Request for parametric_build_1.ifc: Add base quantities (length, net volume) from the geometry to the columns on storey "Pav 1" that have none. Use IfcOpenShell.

First a look at what the model holds.

```python
import ifcopenshell
import ifcopenshell.util.element
import ifcopenshell.util.unit

model = ifcopenshell.open("parametric_build_1.ifc")
print(model.schema)
for unit_type in ("LENGTHUNIT", "AREAUNIT", "VOLUMEUNIT"):
    print(unit_type, ifcopenshell.util.unit.calculate_unit_scale(model, unit_type))
storey = next(s for s in model.by_type("IfcBuildingStorey") if s.Name == "Pav 1")
columns = [e for e in ifcopenshell.util.element.get_decomposition(storey) if e.is_a("IfcColumn")]
for e in sorted(columns, key=lambda e: e.id()):
    print(e.id(), e.is_a(), e.Name, list(ifcopenshell.util.element.get_psets(e, qtos_only=True)), sep=" | ")
```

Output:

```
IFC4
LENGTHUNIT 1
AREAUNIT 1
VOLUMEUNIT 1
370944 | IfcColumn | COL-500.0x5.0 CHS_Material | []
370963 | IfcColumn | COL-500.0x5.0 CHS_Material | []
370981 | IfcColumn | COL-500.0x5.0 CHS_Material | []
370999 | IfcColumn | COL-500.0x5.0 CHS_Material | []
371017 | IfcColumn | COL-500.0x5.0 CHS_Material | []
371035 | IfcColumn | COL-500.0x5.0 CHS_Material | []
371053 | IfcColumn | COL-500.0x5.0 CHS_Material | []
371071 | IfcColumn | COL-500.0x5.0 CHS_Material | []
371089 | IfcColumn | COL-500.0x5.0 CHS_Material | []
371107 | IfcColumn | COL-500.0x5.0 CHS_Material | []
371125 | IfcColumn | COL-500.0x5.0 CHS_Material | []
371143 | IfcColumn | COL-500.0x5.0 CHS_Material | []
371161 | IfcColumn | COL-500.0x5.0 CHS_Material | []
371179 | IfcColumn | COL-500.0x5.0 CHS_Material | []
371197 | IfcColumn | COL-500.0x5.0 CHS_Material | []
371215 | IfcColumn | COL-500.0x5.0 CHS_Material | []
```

```python
import ifcopenshell
import ifcopenshell.api.pset
import ifcopenshell.geom
import ifcopenshell.util.element
import ifcopenshell.util.shape
import ifcopenshell.util.unit

model = ifcopenshell.open("parametric_build_1.ifc")
unit_scale = ifcopenshell.util.unit.calculate_unit_scale(model)
volume_scale = ifcopenshell.util.unit.calculate_unit_scale(model, "VOLUMEUNIT")
settings = ifcopenshell.geom.settings()

storey = next(s for s in model.by_type("IfcBuildingStorey") if s.Name == "Pav 1")
columns = [e for e in ifcopenshell.util.element.get_decomposition(storey) if e.is_a("IfcColumn")]

for e in sorted(columns, key=lambda e: e.id()):
    if ifcopenshell.util.element.get_psets(e, qtos_only=True, should_inherit=False):
        continue
    # Geometry comes back in metres, in the element's own axes.
    shape = ifcopenshell.geom.create_shape(settings, e)
    values = {
        "Length": ifcopenshell.util.shape.get_z(shape.geometry) / unit_scale,
        "NetVolume": ifcopenshell.util.shape.get_volume(shape.geometry) / volume_scale,
    }
    qto = ifcopenshell.api.pset.add_qto(model, product=e, name="Qto_ColumnBaseQuantities")
    ifcopenshell.api.pset.edit_qto(model, qto=qto, properties=values)
    print(e.id(), {k: round(v, 3) for k, v in values.items()})

model.write("parametric_build_1_rev.ifc")
```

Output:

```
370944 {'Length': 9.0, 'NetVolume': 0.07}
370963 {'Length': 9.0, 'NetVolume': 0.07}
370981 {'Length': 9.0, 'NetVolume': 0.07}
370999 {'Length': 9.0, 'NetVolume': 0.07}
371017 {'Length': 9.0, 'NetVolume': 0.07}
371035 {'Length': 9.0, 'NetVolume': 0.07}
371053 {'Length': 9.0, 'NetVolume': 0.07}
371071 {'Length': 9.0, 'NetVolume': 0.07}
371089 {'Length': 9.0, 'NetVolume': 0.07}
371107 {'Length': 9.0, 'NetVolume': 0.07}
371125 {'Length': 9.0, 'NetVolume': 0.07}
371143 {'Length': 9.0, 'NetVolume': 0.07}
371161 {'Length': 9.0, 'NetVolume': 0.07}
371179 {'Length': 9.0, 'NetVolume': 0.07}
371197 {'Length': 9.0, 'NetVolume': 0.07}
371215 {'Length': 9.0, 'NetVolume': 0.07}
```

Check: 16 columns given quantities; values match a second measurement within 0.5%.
